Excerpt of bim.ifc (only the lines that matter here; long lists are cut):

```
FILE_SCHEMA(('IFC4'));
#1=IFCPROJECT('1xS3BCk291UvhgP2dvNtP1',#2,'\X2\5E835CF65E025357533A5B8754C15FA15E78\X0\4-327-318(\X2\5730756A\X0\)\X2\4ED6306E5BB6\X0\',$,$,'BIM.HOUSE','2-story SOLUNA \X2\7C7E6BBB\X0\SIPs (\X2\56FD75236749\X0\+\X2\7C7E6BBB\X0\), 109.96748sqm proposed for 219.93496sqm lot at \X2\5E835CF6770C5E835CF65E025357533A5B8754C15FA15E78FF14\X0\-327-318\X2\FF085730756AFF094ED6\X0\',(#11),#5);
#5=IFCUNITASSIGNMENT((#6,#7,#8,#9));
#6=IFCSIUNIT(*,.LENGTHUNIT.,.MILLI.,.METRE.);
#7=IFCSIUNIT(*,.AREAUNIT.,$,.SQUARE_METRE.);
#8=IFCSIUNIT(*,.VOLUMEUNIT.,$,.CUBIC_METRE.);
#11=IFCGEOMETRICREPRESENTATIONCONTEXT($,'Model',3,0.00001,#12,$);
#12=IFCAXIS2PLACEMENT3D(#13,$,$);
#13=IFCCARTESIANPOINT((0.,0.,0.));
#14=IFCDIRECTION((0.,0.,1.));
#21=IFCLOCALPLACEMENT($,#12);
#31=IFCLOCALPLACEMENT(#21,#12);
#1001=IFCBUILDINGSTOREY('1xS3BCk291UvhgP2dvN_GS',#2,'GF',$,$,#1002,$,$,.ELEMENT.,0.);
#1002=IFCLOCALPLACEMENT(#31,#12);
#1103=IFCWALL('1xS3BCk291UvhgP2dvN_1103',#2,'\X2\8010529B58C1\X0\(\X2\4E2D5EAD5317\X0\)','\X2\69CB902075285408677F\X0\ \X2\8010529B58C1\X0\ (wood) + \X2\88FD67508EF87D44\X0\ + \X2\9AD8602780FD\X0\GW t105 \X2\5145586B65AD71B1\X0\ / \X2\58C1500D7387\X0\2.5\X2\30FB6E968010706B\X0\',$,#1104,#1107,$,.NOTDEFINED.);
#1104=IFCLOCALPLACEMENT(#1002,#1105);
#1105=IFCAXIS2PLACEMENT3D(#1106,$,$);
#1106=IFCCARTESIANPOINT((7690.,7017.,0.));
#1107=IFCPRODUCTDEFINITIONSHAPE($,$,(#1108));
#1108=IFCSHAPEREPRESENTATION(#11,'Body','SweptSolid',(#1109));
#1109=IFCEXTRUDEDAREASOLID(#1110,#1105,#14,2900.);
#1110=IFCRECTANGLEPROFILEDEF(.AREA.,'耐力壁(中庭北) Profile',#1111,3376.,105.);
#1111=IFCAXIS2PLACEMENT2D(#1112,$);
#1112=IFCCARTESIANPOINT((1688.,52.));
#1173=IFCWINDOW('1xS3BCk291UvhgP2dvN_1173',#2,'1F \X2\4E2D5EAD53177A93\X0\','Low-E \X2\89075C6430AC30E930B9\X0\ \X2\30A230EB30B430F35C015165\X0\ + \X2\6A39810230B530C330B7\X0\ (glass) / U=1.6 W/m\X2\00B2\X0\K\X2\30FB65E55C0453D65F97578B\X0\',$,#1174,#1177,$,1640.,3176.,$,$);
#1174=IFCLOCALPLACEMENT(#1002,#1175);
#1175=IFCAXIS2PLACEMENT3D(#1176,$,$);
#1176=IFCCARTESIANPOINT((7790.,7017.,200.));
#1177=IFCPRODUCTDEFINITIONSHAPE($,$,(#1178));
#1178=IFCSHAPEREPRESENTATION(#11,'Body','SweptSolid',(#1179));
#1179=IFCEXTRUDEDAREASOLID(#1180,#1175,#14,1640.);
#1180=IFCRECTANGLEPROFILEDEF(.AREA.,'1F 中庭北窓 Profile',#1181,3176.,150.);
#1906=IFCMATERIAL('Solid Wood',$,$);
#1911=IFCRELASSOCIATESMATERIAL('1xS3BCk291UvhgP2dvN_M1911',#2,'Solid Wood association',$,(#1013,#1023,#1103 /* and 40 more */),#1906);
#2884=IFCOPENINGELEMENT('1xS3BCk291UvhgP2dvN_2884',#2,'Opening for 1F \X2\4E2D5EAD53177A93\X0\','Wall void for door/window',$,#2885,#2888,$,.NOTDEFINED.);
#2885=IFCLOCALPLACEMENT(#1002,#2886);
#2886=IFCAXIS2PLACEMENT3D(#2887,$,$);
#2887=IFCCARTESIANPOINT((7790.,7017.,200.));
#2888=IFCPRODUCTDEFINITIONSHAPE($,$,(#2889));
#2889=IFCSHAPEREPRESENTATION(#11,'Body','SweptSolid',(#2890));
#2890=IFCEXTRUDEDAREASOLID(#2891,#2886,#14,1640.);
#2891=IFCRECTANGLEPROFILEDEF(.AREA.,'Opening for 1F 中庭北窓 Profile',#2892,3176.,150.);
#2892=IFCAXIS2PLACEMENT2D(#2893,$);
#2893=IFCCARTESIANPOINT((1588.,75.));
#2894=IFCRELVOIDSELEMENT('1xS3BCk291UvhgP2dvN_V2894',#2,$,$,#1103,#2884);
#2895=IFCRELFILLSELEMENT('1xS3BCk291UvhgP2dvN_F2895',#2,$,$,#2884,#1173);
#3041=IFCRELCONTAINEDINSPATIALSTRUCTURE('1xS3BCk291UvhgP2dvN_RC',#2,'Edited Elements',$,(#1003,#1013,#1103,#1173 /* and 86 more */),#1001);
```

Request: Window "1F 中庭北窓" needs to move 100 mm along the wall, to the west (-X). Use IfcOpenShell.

```python
import ifcopenshell
import ifcopenshell.api.geometry
import ifcopenshell.util.placement
import ifcopenshell.util.unit

model = ifcopenshell.open("bim.ifc")
unit_scale = ifcopenshell.util.unit.calculate_unit_scale(model)

window = model.by_guid("1xS3BCk291UvhgP2dvN_1173")
opening = window.FillsVoids[0].RelatingOpeningElement
wall = opening.VoidsElements[0].RelatingBuildingElement

wall_matrix = ifcopenshell.util.placement.get_local_placement(wall.ObjectPlacement)
shift = wall_matrix[:3, 0] * -0.1 / unit_scale
before = ifcopenshell.util.placement.get_local_placement(window.ObjectPlacement)[:3, 3].copy()

# The window is not placed relative to its opening, so move both.
for product in (opening, window):
    matrix = ifcopenshell.util.placement.get_local_placement(product.ObjectPlacement)
    matrix[:3, 3] += shift
    ifcopenshell.api.geometry.edit_object_placement(model, product=product, matrix=matrix, is_si=False)

after = ifcopenshell.util.placement.get_local_placement(window.ObjectPlacement)[:3, 3]
print("window moved by", (after - before).round(3) + 0.0)

model.write("bim_edited.ifc")
```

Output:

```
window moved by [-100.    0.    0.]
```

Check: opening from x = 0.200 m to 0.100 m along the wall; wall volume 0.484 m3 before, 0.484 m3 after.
